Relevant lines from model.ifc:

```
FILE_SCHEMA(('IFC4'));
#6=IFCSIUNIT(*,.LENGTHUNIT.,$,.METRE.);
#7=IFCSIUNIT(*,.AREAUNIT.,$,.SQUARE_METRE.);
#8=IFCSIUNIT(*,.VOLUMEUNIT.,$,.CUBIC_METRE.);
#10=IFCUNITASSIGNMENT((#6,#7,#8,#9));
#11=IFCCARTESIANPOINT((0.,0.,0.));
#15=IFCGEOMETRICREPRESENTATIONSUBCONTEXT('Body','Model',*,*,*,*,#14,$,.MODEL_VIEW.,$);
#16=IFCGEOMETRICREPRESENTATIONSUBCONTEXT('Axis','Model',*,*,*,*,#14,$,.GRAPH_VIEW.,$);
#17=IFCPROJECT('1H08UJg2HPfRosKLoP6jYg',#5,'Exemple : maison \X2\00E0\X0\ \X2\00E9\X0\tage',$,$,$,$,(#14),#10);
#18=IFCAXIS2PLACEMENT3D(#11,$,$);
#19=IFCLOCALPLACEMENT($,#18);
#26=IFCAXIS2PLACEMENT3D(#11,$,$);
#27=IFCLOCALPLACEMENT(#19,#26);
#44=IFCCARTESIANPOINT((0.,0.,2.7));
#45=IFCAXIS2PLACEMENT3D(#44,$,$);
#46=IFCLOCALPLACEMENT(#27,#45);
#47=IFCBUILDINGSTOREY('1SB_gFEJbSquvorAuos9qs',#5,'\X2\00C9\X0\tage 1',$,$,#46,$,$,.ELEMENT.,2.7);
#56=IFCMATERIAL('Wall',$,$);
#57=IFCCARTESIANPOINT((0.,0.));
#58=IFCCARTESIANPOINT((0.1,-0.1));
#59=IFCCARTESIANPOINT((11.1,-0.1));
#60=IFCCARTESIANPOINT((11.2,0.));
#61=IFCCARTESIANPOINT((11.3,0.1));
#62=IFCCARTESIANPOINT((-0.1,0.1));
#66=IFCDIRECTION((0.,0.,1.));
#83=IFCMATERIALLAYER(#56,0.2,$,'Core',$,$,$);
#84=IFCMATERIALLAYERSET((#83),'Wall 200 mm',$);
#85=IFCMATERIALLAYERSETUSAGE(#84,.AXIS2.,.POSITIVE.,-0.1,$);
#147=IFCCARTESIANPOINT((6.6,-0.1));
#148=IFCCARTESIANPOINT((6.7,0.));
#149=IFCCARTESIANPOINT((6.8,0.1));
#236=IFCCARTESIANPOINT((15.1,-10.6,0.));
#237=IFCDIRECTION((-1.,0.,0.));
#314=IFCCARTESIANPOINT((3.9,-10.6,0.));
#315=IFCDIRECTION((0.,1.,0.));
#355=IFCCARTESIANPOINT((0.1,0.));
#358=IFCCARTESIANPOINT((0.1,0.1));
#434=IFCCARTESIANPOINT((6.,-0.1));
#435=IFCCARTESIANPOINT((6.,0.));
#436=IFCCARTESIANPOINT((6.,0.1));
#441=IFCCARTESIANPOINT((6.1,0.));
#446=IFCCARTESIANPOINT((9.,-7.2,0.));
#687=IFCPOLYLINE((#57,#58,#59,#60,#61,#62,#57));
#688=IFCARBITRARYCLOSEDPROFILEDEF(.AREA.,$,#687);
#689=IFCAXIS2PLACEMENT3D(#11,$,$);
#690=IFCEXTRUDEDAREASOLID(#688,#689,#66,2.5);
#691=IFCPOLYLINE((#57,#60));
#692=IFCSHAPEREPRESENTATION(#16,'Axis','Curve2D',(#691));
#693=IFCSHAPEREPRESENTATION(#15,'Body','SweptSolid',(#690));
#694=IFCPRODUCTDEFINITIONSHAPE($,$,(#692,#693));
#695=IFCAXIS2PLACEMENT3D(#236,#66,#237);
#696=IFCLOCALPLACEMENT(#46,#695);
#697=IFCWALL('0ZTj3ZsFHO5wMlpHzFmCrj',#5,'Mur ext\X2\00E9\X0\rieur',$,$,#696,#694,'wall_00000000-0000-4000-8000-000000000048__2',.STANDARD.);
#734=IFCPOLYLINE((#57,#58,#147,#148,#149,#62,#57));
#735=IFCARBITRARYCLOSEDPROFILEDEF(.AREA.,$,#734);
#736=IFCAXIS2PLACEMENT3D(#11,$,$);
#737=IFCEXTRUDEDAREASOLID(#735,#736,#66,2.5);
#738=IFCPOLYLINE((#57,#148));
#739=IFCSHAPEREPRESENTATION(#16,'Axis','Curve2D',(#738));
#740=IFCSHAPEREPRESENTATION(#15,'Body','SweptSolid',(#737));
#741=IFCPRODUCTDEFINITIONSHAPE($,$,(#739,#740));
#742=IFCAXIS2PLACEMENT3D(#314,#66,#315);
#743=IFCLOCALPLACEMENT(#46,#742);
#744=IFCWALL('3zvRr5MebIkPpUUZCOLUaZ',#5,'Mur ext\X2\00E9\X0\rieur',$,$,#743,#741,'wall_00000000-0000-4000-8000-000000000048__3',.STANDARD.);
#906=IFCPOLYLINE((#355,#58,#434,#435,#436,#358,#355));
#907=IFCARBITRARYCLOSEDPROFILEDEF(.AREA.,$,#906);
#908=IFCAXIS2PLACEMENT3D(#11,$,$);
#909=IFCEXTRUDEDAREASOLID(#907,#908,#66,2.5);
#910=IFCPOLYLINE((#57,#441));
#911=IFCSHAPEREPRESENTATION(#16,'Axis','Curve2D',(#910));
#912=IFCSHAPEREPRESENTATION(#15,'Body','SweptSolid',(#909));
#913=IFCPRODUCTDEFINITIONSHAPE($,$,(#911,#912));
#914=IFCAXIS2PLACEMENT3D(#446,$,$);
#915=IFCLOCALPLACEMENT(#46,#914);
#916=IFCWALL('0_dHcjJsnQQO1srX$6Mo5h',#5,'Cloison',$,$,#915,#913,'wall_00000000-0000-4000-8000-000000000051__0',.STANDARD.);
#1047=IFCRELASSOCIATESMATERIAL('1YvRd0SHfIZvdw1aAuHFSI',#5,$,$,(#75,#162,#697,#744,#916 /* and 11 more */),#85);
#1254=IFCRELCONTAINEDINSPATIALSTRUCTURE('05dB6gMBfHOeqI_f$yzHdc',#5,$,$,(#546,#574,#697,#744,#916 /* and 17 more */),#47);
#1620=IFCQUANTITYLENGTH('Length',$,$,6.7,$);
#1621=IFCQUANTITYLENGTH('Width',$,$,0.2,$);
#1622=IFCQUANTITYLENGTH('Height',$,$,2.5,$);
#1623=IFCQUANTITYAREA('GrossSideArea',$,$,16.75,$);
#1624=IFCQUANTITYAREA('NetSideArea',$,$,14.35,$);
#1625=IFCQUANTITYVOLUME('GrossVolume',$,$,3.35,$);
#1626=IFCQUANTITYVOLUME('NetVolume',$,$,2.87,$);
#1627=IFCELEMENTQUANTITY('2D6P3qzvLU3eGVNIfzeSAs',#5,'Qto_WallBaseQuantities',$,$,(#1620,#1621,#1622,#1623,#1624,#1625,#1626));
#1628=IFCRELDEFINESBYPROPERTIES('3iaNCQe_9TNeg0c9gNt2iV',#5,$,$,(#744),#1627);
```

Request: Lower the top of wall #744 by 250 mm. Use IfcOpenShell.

```python
import ifcopenshell
import ifcopenshell.api.pset
import ifcopenshell.geom
import ifcopenshell.util.element
import ifcopenshell.util.representation
import ifcopenshell.util.shape
import ifcopenshell.util.unit

model = ifcopenshell.open("model.ifc")
unit_scale = ifcopenshell.util.unit.calculate_unit_scale(model)
area_scale = ifcopenshell.util.unit.calculate_unit_scale(model, "AREAUNIT")
volume_scale = ifcopenshell.util.unit.calculate_unit_scale(model, "VOLUMEUNIT")
settings = ifcopenshell.geom.settings()


def volume(element):
    """Net volume in cubic metres, openings subtracted."""
    shape = ifcopenshell.geom.create_shape(settings, element)
    return ifcopenshell.util.shape.get_volume(shape.geometry)


wall = model.by_id(744)
before = volume(wall)

body = ifcopenshell.util.representation.get_representation(wall, "Model", "Body")
solid = body.Items[0]
old_height = solid.Depth
solid.Depth -= 0.25 / unit_scale
after = volume(wall)
thickness = 0.2  # wall thickness in metres

# Update the stored height, areas and volumes.
qto = model.by_id(ifcopenshell.util.element.get_pset(wall, "Qto_WallBaseQuantities", should_inherit=False)["id"])
ifcopenshell.api.pset.edit_qto(model, qto=qto, properties={
    "Height": solid.Depth,
    "GrossSideArea": ifcopenshell.util.element.get_pset(wall, "Qto_WallBaseQuantities", "GrossSideArea") * solid.Depth / old_height,
    "NetSideArea": after / thickness / area_scale,
    "GrossVolume": ifcopenshell.util.element.get_pset(wall, "Qto_WallBaseQuantities", "GrossVolume") * solid.Depth / old_height,
    "NetVolume": after / volume_scale,
})

print(f"height {old_height:g} -> {solid.Depth:g}, volume {before:.3f} -> {after:.3f} m3")

model.write("model_v2.ifc")
```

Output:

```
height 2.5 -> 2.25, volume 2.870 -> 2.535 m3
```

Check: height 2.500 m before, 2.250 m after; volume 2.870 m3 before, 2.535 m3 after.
